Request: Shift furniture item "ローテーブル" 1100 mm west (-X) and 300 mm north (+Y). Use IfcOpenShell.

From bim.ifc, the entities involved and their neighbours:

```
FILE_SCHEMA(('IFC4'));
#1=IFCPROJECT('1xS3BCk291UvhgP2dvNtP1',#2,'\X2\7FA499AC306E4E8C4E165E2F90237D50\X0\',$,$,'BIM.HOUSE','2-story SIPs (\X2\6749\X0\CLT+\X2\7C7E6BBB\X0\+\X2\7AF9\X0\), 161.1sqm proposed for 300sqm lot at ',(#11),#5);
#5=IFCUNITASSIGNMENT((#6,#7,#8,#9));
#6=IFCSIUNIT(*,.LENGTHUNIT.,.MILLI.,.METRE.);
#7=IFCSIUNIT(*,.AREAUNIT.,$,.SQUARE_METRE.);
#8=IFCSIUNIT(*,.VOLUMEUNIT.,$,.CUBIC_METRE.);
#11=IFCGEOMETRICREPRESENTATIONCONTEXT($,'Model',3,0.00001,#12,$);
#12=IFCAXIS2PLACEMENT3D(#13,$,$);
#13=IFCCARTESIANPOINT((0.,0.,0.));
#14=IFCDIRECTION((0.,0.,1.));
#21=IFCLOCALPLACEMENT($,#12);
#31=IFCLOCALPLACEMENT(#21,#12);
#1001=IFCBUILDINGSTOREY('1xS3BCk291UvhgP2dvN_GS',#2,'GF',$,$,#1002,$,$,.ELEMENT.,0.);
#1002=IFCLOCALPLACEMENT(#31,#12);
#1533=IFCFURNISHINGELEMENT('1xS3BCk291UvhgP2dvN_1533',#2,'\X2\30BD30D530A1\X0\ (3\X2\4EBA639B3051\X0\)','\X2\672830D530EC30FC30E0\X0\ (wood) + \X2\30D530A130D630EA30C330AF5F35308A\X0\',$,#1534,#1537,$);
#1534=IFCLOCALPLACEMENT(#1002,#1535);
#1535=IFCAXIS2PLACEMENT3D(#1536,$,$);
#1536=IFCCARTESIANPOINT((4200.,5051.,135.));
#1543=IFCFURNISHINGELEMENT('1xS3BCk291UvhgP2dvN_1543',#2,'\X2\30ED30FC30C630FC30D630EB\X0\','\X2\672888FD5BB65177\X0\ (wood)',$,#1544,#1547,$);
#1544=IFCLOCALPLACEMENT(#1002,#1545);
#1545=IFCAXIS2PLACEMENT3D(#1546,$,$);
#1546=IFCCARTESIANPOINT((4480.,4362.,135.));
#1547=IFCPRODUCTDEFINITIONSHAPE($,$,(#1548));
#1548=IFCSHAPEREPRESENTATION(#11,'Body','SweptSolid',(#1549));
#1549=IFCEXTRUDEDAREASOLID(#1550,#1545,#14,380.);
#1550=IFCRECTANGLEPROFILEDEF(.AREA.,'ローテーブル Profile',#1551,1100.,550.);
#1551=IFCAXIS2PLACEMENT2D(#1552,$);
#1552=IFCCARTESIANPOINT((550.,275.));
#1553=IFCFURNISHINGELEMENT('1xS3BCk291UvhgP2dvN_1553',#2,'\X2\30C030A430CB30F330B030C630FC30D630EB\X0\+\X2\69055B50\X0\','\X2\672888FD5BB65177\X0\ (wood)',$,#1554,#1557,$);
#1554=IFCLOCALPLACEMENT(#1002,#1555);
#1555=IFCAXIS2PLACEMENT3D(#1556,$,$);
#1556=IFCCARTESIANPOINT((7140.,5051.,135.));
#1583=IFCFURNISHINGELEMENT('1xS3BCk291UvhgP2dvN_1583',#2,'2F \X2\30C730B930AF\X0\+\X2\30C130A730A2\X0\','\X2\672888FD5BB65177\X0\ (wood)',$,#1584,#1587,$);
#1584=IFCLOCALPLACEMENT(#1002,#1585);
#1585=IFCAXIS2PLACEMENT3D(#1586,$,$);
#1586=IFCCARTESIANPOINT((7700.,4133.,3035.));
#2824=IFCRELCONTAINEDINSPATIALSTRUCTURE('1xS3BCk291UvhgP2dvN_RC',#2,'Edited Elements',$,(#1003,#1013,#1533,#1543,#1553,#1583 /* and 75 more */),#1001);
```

```python
import ifcopenshell
import ifcopenshell.api.geometry
import ifcopenshell.util.placement

model = ifcopenshell.open("bim.ifc")

item = model.by_guid("1xS3BCk291UvhgP2dvN_1543")
matrix = ifcopenshell.util.placement.get_local_placement(item.ObjectPlacement)
matrix[0, 3] -= 1100.0
matrix[1, 3] += 300.0
ifcopenshell.api.geometry.edit_object_placement(model, product=item, matrix=matrix, is_si=False)

print(ifcopenshell.util.placement.get_local_placement(item.ObjectPlacement).round(3) + 0.0)

model.write("bim_edited.ifc")
```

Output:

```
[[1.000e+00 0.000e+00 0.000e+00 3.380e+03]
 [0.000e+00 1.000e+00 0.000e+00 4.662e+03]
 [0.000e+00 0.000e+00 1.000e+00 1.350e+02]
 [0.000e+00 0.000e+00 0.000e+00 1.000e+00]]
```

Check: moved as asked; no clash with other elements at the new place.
